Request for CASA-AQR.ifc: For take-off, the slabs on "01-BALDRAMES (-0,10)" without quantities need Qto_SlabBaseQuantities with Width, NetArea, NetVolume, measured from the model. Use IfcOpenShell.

First a look at what the model holds.

```python
import ifcopenshell
import ifcopenshell.util.element
import ifcopenshell.util.unit

model = ifcopenshell.open("CASA-AQR.ifc")
print(model.schema)
for unit_type in ("LENGTHUNIT", "AREAUNIT", "VOLUMEUNIT"):
    print(unit_type, ifcopenshell.util.unit.calculate_unit_scale(model, unit_type))
storey = next(s for s in model.by_type("IfcBuildingStorey") if s.Name == "01-BALDRAMES (-0,10)")
slabs = [e for e in ifcopenshell.util.element.get_decomposition(storey) if e.is_a("IfcSlab")]
for e in sorted(slabs, key=lambda e: e.id()):
    print(e.id(), e.is_a(), e.Name, list(ifcopenshell.util.element.get_psets(e, qtos_only=True)), sep=" | ")
```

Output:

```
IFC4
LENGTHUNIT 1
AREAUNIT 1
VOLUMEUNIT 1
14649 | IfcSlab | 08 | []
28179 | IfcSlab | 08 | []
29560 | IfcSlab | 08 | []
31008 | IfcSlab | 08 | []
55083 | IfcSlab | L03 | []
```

```python
import ifcopenshell
import ifcopenshell.api.pset
import ifcopenshell.geom
import ifcopenshell.util.element
import ifcopenshell.util.shape
import ifcopenshell.util.unit

model = ifcopenshell.open("CASA-AQR.ifc")
unit_scale = ifcopenshell.util.unit.calculate_unit_scale(model)
area_scale = ifcopenshell.util.unit.calculate_unit_scale(model, "AREAUNIT")
volume_scale = ifcopenshell.util.unit.calculate_unit_scale(model, "VOLUMEUNIT")
settings = ifcopenshell.geom.settings()

storey = next(s for s in model.by_type("IfcBuildingStorey") if s.Name == "01-BALDRAMES (-0,10)")
slabs = [e for e in ifcopenshell.util.element.get_decomposition(storey) if e.is_a("IfcSlab")]

for e in sorted(slabs, key=lambda e: e.id()):
    if ifcopenshell.util.element.get_psets(e, qtos_only=True, should_inherit=False):
        continue
    # Geometry comes back in metres, in the element's own axes.
    shape = ifcopenshell.geom.create_shape(settings, e)
    values = {
        "Width": ifcopenshell.util.shape.get_z(shape.geometry) / unit_scale,
        "NetArea": ifcopenshell.util.shape.get_footprint_area(shape.geometry) / area_scale,
        "NetVolume": ifcopenshell.util.shape.get_volume(shape.geometry) / volume_scale,
    }
    qto = ifcopenshell.api.pset.add_qto(model, product=e, name="Qto_SlabBaseQuantities")
    ifcopenshell.api.pset.edit_qto(model, qto=qto, properties=values)
    print(e.id(), {k: round(v, 3) for k, v in values.items()})

model.write("CASA-AQR_rev.ifc")
```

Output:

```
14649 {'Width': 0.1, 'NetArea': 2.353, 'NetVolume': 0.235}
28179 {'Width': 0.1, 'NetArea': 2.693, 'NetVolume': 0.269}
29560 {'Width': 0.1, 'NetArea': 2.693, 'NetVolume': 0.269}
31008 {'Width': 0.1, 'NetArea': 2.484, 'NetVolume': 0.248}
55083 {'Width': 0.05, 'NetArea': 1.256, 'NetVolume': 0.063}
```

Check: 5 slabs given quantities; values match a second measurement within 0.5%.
